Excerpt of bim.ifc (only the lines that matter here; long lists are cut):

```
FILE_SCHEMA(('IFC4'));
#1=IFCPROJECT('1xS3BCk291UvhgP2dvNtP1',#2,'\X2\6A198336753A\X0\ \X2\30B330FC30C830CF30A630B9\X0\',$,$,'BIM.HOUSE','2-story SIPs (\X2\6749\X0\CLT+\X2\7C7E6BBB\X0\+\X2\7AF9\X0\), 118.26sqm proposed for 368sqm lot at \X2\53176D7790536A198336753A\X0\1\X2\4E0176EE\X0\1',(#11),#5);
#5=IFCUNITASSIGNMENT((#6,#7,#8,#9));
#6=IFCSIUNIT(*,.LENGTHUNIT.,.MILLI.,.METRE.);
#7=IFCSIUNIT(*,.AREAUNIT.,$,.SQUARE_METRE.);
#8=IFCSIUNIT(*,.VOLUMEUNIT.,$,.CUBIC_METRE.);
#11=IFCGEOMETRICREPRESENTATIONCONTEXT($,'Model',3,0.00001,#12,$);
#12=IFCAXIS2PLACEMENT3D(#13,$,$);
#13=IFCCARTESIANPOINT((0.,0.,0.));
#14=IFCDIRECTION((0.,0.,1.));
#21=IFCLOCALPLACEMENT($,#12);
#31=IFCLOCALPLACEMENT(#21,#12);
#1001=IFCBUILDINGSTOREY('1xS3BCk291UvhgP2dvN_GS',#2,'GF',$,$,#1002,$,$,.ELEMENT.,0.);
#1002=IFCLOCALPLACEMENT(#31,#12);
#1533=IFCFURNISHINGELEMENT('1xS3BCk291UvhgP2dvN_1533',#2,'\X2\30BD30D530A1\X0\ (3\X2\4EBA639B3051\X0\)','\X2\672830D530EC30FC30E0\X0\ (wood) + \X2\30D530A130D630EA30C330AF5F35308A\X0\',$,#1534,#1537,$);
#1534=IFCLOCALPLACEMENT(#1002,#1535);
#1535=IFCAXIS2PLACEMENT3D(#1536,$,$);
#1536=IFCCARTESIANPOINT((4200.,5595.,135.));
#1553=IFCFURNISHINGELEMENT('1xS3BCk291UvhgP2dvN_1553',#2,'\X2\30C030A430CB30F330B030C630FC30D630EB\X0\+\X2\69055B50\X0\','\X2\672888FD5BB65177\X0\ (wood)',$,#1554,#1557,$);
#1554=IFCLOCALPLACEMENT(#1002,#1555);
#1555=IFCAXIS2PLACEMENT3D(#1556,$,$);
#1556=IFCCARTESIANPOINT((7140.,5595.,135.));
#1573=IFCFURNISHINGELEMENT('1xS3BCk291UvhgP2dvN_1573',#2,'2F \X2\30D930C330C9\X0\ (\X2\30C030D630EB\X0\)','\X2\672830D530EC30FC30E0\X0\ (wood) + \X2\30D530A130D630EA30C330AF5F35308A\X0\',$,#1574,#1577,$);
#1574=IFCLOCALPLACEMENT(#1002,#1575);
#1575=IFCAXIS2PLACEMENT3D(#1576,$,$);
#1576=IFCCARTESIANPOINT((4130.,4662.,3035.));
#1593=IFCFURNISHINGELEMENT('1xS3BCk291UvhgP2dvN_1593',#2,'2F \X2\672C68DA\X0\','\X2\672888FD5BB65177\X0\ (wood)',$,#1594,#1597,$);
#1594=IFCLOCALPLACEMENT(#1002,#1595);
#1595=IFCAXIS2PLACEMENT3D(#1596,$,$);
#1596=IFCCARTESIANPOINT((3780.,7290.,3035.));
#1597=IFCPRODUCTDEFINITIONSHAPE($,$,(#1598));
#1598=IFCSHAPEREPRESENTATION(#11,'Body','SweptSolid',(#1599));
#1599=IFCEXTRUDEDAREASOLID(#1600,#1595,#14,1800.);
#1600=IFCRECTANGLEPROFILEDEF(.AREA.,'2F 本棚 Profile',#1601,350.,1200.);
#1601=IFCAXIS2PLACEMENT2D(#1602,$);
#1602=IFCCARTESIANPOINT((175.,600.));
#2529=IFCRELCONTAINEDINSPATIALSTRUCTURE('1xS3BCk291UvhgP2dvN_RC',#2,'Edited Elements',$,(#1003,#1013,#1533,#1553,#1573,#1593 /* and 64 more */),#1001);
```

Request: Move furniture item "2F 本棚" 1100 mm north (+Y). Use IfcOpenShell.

```python
import ifcopenshell
import ifcopenshell.api.geometry
import ifcopenshell.util.placement
import ifcopenshell.util.unit

model = ifcopenshell.open("bim.ifc")
unit_scale = ifcopenshell.util.unit.calculate_unit_scale(model)

item = model.by_guid("1xS3BCk291UvhgP2dvN_1593")
matrix = ifcopenshell.util.placement.get_local_placement(item.ObjectPlacement)
matrix[1, 3] += 1.1 / unit_scale
ifcopenshell.api.geometry.edit_object_placement(model, product=item, matrix=matrix, is_si=False)

print(ifcopenshell.util.placement.get_local_placement(item.ObjectPlacement).round(3) + 0.0)

model.write("bim_updated.ifc")
```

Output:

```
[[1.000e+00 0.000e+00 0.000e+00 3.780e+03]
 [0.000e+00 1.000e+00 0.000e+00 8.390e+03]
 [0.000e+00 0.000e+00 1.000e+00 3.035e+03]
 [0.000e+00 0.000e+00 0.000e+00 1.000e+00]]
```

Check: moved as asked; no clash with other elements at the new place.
